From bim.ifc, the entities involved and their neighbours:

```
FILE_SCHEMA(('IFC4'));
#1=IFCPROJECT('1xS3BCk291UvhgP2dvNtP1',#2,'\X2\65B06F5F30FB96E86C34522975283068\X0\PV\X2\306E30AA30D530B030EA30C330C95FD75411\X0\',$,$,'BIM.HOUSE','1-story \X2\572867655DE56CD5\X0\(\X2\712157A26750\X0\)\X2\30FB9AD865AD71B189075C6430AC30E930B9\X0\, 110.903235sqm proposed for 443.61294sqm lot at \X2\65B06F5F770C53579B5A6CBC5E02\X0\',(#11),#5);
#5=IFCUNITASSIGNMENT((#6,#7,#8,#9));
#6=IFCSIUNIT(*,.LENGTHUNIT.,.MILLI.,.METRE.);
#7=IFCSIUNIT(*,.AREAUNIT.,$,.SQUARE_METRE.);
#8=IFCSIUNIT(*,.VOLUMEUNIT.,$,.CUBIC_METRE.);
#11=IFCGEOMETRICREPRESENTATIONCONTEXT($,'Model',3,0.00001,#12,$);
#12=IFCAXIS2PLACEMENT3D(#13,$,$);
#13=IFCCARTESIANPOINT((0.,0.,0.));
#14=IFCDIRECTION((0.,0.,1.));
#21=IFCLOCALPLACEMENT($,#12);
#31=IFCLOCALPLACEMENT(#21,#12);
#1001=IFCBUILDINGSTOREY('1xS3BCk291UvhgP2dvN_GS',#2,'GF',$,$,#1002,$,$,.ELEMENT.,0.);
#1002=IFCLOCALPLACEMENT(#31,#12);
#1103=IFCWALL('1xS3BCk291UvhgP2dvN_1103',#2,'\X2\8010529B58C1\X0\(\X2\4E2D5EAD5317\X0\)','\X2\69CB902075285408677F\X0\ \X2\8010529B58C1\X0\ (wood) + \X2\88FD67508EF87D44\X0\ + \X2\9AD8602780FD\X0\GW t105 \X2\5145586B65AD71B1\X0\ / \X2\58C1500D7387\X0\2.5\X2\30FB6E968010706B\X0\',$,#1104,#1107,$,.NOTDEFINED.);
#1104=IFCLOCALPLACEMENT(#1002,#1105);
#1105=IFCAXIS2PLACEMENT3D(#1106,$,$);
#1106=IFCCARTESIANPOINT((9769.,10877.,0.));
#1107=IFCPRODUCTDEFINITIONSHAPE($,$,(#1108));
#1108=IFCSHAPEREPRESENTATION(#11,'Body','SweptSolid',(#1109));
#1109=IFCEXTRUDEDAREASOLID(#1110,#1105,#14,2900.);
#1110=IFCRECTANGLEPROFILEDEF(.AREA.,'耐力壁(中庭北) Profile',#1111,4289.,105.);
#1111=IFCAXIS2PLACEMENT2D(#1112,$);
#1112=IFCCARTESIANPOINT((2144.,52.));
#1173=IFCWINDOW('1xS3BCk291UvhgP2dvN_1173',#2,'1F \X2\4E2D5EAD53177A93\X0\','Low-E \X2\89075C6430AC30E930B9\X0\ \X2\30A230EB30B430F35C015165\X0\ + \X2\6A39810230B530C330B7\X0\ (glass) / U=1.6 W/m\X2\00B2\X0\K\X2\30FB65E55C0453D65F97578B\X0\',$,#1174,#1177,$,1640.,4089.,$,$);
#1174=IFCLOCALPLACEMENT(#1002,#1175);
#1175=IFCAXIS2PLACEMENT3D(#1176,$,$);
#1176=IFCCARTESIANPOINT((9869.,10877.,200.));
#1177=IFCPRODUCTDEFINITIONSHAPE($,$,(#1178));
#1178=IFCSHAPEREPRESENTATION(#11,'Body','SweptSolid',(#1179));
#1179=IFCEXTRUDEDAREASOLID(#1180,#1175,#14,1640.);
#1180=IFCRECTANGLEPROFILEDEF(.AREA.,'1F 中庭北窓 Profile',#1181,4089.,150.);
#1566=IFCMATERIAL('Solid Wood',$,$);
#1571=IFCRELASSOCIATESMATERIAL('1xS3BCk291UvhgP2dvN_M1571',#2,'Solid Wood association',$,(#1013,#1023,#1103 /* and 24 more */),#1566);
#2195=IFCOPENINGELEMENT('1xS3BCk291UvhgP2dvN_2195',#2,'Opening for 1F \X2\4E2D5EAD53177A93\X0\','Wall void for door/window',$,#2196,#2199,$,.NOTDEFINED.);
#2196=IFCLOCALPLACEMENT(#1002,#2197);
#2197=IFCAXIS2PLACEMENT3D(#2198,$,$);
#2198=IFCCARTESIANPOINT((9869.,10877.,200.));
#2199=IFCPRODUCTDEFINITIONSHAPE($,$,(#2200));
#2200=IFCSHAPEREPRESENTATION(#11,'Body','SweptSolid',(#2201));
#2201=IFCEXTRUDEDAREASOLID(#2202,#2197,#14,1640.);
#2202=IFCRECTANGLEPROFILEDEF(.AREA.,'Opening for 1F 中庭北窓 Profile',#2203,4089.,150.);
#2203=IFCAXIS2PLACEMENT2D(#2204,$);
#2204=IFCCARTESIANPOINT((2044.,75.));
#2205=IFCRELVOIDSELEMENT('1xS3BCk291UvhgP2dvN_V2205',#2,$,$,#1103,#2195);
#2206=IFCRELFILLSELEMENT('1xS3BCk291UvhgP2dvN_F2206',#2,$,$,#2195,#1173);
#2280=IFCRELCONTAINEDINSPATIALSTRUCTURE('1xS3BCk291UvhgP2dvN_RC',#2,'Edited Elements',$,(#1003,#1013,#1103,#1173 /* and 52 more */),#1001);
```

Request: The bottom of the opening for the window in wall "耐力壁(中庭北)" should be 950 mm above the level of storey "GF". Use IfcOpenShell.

```python
import numpy as np
import ifcopenshell
import ifcopenshell.api.geometry
import ifcopenshell.geom
import ifcopenshell.util.element
import ifcopenshell.util.placement
import ifcopenshell.util.shape
import ifcopenshell.util.unit

model = ifcopenshell.open("bim.ifc")
unit_scale = ifcopenshell.util.unit.calculate_unit_scale(model)

window = model.by_id(1173)
opening = window.FillsVoids[0].RelatingOpeningElement
storey = ifcopenshell.util.element.get_container(window, ifc_class="IfcBuildingStorey")
level = ifcopenshell.util.placement.get_local_placement(storey.ObjectPlacement)[2, 3]

# The opening's origin need not be at the sill, so measure its lowest point.
shape = ifcopenshell.geom.create_shape(ifcopenshell.geom.settings(), opening)
bottom = ifcopenshell.util.shape.get_shape_bottom_elevation(shape, shape.geometry) / unit_scale
dz = level + 0.95 / unit_scale - bottom

shift = np.array([0.0, 0.0, dz])
# The window is not placed relative to its opening, so move both.
for product in (opening, window):
    matrix = ifcopenshell.util.placement.get_local_placement(product.ObjectPlacement)
    matrix[:3, 3] += shift
    ifcopenshell.api.geometry.edit_object_placement(model, product=product, matrix=matrix, is_si=False)

print(f"moved by {dz * unit_scale:+.3f} m")

model.write("bim_edited.ifc")
```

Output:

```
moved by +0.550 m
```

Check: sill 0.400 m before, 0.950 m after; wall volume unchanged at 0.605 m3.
